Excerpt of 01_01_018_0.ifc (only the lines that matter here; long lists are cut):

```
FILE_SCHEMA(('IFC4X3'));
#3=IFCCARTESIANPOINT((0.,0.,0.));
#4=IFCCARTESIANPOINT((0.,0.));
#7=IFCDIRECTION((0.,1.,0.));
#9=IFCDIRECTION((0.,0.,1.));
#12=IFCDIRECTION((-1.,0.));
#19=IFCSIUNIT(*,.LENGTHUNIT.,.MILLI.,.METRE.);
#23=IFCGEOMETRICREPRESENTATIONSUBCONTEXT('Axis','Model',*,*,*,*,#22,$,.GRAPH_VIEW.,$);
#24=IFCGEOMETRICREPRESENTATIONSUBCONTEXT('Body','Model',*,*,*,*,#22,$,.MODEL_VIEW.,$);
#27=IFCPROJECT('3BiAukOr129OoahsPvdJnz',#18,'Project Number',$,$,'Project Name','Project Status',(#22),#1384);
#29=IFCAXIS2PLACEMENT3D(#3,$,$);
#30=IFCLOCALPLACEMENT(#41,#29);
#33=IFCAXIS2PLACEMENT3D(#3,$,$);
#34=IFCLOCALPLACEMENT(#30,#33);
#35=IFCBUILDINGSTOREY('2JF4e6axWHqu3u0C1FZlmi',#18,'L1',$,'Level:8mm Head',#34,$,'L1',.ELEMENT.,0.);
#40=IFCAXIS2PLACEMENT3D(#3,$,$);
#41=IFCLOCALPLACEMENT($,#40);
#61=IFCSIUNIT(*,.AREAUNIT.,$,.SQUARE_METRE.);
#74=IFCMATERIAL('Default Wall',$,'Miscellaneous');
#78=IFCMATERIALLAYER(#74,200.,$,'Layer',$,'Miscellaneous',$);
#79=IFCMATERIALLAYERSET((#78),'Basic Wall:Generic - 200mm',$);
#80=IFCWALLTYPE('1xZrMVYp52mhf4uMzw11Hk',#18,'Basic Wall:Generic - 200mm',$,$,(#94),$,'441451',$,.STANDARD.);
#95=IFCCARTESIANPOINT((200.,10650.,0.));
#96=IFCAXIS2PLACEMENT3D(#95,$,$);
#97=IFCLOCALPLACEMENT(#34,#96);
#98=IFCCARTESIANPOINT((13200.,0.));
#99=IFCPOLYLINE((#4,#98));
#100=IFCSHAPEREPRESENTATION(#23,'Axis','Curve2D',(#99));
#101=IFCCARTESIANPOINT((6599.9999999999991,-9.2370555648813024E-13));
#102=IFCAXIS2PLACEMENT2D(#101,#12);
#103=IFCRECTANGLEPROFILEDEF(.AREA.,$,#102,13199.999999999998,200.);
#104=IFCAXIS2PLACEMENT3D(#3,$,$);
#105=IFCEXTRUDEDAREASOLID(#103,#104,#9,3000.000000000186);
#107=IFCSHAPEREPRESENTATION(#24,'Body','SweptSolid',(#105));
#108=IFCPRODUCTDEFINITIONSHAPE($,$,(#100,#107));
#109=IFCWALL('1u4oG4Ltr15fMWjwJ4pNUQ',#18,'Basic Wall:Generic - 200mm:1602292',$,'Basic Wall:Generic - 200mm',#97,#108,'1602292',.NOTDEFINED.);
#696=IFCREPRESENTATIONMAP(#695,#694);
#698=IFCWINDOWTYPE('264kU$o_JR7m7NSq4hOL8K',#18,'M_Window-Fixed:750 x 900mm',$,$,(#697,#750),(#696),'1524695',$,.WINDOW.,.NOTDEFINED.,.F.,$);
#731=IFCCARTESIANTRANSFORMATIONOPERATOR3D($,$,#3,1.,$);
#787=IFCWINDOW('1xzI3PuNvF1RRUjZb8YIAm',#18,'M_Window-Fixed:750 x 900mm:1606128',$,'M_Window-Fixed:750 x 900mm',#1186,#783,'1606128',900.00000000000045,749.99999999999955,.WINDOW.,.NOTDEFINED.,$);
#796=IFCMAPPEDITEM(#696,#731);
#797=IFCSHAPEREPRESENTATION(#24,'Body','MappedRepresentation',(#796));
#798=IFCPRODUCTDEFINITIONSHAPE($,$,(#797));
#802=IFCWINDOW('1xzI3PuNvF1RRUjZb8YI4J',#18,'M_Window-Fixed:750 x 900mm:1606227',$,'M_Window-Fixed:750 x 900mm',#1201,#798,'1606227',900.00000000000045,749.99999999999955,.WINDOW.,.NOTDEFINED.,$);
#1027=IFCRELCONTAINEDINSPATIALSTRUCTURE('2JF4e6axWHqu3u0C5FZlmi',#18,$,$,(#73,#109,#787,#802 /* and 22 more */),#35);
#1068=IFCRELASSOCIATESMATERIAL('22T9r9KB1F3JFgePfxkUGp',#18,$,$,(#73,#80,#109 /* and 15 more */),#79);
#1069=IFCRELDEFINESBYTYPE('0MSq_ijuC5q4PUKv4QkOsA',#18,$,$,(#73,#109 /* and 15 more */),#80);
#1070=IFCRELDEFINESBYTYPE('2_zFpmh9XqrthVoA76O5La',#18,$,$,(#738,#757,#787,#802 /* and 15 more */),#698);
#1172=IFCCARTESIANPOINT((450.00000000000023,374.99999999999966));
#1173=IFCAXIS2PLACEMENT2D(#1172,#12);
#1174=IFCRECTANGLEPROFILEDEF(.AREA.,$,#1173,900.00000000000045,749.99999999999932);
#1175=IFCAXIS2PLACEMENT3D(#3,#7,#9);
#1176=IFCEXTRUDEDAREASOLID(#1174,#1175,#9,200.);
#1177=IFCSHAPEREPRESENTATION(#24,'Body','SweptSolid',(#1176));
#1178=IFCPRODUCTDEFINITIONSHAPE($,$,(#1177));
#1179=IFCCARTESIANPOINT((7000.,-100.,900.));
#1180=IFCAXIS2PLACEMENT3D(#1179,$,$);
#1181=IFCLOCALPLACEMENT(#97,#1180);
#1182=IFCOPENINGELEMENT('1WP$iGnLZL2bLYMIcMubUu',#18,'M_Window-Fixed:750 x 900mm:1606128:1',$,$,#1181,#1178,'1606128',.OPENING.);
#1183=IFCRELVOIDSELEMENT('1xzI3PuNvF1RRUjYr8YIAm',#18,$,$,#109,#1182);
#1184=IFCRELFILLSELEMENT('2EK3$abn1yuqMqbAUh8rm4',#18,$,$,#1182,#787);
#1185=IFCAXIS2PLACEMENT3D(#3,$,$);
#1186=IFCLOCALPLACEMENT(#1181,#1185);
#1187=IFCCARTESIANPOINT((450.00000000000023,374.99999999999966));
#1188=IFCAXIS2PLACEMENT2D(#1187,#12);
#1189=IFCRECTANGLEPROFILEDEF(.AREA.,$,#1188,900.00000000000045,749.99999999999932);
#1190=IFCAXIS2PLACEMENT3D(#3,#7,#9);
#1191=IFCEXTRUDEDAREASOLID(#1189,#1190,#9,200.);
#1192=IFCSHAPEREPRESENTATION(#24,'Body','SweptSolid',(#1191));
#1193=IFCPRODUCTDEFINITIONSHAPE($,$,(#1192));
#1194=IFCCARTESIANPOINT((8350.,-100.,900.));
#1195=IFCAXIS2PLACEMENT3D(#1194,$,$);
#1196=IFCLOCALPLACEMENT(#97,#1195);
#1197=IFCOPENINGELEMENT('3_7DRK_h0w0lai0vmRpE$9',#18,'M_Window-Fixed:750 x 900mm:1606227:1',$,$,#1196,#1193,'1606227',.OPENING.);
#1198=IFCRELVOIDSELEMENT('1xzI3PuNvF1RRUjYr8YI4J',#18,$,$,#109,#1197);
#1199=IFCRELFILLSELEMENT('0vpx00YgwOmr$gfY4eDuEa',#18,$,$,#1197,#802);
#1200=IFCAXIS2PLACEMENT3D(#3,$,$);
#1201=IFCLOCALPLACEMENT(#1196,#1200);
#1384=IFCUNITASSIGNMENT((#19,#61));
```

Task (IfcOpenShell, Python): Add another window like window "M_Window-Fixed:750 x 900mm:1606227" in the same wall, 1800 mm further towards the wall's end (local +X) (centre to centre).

```python
import ifcopenshell
import ifcopenshell.api.feature
import ifcopenshell.api.geometry
import ifcopenshell.api.root
import ifcopenshell.geom
import ifcopenshell.util.element
import ifcopenshell.util.placement
import ifcopenshell.util.shape
import ifcopenshell.util.unit

model = ifcopenshell.open("01_01_018_0.ifc")
unit_scale = ifcopenshell.util.unit.calculate_unit_scale(model)
settings = ifcopenshell.geom.settings()


def volume(element):
    """Net volume in cubic metres, openings subtracted."""
    shape = ifcopenshell.geom.create_shape(settings, element)
    return ifcopenshell.util.shape.get_volume(shape.geometry)


def reuse_history(source, copy):
    """copy_class also copies each property set's owner history, people and application; keep the originals."""
    for rel in copy.IsDefinedBy:
        if rel.is_a("IfcRelDefinesByProperties") and (history := rel.RelatingPropertyDefinition.OwnerHistory):
            rel.RelatingPropertyDefinition.OwnerHistory = source.OwnerHistory
            ifcopenshell.util.element.remove_deep2(model, history)


window = model.by_guid("1xzI3PuNvF1RRUjZb8YI4J")
opening = window.FillsVoids[0].RelatingOpeningElement
wall = opening.VoidsElements[0].RelatingBuildingElement
before = volume(wall)
shift = ifcopenshell.util.placement.get_local_placement(wall.ObjectPlacement)[:3, 0] * 1.8 / unit_scale

# copy_class copies the void relationship, type, container and properties, but no geometry.
new_opening = ifcopenshell.api.root.copy_class(model, product=opening)
new_opening.Representation = ifcopenshell.util.element.copy_deep(
    model, opening.Representation, exclude=["IfcGeometricRepresentationContext", "IfcRepresentationMap"]
)
new_opening.Name = "M_Window-Fixed:750 x 900mm"
new_opening.Tag = None
new_window = ifcopenshell.api.root.copy_class(model, product=window)
new_window.Representation = ifcopenshell.util.element.copy_deep(
    model, window.Representation, exclude=["IfcGeometricRepresentationContext", "IfcRepresentationMap"]
)
new_window.Name = "M_Window-Fixed:750 x 900mm"
new_window.Tag = None
reuse_history(window, new_window)
ifcopenshell.api.feature.add_filling(model, opening=new_opening, element=new_window)

for old, new in ((opening, new_opening), (window, new_window)):
    matrix = ifcopenshell.util.placement.get_local_placement(old.ObjectPlacement)
    matrix[:3, 3] += shift
    ifcopenshell.api.geometry.edit_object_placement(model, product=new, matrix=matrix, is_si=False)

after = volume(wall)

print(f"wall volume {before:.3f} -> {after:.3f} m3")

model.write("01_01_018_0_v2.ifc")
```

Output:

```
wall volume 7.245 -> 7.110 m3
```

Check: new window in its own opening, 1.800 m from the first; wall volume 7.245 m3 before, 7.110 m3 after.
